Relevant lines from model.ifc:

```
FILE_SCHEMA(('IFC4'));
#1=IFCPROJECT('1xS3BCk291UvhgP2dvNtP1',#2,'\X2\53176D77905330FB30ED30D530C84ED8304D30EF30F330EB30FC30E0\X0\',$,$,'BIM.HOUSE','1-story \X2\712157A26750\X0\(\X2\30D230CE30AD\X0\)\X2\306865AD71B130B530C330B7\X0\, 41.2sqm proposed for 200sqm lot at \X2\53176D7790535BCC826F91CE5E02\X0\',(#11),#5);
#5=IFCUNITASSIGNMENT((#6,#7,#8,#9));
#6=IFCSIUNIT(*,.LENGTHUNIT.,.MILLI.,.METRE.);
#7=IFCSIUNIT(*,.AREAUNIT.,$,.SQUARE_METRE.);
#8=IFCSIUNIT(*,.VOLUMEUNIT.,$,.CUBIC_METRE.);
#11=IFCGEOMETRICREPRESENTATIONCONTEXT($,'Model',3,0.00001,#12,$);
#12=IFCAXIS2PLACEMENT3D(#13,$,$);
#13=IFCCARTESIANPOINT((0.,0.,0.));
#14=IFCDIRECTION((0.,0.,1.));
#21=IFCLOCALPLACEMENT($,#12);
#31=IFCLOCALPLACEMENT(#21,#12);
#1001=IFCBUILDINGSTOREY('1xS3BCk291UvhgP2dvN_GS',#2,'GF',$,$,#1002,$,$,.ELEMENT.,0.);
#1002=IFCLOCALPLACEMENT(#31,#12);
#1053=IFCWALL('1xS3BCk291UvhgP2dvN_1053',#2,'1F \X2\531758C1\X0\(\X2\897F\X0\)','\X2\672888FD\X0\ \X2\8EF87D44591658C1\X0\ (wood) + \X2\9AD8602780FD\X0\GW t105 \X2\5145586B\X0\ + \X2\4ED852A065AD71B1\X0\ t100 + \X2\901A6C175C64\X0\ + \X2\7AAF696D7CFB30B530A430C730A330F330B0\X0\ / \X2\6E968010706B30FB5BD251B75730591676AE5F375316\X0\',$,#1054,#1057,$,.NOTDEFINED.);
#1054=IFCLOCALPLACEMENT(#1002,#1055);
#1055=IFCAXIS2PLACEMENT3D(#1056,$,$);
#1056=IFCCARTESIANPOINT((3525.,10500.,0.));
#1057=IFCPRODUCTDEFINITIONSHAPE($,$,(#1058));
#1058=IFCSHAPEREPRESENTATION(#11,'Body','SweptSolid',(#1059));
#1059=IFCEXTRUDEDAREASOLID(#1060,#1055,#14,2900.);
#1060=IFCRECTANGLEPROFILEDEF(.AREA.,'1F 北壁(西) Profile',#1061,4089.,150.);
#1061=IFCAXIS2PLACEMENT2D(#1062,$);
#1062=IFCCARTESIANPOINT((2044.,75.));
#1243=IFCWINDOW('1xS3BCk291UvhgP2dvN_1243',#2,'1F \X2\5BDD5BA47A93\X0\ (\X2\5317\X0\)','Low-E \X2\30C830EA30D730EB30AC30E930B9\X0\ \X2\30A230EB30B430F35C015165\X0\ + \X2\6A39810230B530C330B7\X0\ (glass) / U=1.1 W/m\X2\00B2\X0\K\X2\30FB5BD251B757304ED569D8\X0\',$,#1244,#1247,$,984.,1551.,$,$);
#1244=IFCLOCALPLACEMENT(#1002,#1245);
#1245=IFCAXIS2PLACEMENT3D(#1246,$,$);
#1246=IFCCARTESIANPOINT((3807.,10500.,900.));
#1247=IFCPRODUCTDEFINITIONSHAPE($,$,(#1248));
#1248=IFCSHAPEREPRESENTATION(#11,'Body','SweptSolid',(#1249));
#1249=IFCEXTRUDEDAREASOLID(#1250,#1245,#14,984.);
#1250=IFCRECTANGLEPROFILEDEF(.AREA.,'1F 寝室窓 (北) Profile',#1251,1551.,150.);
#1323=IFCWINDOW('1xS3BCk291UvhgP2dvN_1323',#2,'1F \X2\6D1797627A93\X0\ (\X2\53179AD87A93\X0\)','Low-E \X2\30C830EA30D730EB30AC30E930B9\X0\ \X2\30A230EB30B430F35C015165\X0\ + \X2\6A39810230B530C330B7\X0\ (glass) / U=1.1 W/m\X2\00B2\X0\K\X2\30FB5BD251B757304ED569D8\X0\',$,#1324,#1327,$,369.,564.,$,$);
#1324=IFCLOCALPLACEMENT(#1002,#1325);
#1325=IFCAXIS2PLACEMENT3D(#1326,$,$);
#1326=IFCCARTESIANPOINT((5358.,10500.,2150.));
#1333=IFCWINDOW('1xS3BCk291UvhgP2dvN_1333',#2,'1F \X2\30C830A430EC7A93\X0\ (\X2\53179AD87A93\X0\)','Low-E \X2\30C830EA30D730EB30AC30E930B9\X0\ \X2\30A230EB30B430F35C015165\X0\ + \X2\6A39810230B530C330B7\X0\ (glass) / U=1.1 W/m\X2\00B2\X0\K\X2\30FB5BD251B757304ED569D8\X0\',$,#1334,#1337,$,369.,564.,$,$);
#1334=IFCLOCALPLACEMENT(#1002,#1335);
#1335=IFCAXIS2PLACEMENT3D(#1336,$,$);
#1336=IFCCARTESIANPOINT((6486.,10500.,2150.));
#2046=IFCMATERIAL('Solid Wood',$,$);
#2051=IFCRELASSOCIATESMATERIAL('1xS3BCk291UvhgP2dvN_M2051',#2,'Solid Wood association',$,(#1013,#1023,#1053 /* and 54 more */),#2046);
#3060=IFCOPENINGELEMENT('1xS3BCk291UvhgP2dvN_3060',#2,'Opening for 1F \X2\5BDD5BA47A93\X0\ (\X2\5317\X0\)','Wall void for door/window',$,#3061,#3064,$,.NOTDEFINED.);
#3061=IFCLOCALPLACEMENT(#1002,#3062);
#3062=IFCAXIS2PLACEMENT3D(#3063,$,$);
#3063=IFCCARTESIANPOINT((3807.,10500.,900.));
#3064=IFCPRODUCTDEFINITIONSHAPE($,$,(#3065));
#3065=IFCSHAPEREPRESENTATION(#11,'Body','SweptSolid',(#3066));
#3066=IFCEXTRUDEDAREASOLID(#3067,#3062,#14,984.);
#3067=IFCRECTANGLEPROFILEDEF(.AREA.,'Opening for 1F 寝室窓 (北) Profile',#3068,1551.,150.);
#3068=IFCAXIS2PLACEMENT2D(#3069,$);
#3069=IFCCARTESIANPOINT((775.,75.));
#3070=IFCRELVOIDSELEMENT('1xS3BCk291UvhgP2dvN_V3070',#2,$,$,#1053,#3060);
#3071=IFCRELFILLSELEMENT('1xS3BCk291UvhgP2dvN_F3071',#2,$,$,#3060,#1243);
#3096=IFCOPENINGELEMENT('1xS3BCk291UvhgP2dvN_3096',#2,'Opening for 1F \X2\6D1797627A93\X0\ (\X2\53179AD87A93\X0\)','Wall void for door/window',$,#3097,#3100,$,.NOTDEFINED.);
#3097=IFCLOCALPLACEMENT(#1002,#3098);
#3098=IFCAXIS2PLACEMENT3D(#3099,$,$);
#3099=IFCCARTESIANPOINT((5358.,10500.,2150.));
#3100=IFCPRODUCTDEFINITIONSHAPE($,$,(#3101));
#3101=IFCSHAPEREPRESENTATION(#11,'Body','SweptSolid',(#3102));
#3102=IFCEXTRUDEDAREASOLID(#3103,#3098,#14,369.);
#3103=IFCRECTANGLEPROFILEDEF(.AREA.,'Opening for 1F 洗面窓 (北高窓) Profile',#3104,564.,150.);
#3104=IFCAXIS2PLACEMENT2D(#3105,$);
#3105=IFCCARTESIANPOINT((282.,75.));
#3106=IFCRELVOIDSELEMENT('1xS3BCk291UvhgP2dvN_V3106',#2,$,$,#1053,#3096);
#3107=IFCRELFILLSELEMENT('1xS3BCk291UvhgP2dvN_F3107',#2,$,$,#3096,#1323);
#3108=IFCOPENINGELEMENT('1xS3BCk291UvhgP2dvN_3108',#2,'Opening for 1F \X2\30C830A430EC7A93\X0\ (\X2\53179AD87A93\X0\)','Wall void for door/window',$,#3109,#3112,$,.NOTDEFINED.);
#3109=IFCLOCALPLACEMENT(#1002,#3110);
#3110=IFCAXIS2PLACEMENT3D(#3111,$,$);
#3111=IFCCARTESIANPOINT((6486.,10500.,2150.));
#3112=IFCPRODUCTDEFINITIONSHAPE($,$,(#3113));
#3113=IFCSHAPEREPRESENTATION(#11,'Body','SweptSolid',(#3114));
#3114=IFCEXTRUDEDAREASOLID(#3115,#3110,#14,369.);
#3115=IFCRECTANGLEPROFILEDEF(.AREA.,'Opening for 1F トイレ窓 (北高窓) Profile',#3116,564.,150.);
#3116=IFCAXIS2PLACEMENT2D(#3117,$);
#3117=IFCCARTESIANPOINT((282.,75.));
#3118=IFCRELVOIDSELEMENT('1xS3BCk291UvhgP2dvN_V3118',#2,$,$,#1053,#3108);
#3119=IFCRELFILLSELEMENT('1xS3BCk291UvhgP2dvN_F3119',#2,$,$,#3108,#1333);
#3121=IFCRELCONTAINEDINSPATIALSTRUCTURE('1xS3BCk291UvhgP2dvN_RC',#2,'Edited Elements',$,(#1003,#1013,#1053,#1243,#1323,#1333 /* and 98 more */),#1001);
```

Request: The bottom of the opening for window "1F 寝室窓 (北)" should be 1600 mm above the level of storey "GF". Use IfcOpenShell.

```python
import numpy as np
import ifcopenshell
import ifcopenshell.api.geometry
import ifcopenshell.geom
import ifcopenshell.util.element
import ifcopenshell.util.placement
import ifcopenshell.util.shape
import ifcopenshell.util.unit

model = ifcopenshell.open("model.ifc")
unit_scale = ifcopenshell.util.unit.calculate_unit_scale(model)

window = model.by_id(1243)
opening = window.FillsVoids[0].RelatingOpeningElement
storey = ifcopenshell.util.element.get_container(window, ifc_class="IfcBuildingStorey")
level = ifcopenshell.util.placement.get_local_placement(storey.ObjectPlacement)[2, 3]

# The opening's origin need not be at the sill, so measure its lowest point.
shape = ifcopenshell.geom.create_shape(ifcopenshell.geom.settings(), opening)
bottom = ifcopenshell.util.shape.get_shape_bottom_elevation(shape, shape.geometry) / unit_scale
dz = level + 1600.0 - bottom

shift = np.array([0.0, 0.0, dz])
# The window is not placed relative to its opening, so move both.
for product in (opening, window):
    matrix = ifcopenshell.util.placement.get_local_placement(product.ObjectPlacement)
    matrix[:3, 3] += shift
    ifcopenshell.api.geometry.edit_object_placement(model, product=product, matrix=matrix, is_si=False)

print(f"moved by {dz * unit_scale:+.3f} m")

model.write("model_edited.ifc")
```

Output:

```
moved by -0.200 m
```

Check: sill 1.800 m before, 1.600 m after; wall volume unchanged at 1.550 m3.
